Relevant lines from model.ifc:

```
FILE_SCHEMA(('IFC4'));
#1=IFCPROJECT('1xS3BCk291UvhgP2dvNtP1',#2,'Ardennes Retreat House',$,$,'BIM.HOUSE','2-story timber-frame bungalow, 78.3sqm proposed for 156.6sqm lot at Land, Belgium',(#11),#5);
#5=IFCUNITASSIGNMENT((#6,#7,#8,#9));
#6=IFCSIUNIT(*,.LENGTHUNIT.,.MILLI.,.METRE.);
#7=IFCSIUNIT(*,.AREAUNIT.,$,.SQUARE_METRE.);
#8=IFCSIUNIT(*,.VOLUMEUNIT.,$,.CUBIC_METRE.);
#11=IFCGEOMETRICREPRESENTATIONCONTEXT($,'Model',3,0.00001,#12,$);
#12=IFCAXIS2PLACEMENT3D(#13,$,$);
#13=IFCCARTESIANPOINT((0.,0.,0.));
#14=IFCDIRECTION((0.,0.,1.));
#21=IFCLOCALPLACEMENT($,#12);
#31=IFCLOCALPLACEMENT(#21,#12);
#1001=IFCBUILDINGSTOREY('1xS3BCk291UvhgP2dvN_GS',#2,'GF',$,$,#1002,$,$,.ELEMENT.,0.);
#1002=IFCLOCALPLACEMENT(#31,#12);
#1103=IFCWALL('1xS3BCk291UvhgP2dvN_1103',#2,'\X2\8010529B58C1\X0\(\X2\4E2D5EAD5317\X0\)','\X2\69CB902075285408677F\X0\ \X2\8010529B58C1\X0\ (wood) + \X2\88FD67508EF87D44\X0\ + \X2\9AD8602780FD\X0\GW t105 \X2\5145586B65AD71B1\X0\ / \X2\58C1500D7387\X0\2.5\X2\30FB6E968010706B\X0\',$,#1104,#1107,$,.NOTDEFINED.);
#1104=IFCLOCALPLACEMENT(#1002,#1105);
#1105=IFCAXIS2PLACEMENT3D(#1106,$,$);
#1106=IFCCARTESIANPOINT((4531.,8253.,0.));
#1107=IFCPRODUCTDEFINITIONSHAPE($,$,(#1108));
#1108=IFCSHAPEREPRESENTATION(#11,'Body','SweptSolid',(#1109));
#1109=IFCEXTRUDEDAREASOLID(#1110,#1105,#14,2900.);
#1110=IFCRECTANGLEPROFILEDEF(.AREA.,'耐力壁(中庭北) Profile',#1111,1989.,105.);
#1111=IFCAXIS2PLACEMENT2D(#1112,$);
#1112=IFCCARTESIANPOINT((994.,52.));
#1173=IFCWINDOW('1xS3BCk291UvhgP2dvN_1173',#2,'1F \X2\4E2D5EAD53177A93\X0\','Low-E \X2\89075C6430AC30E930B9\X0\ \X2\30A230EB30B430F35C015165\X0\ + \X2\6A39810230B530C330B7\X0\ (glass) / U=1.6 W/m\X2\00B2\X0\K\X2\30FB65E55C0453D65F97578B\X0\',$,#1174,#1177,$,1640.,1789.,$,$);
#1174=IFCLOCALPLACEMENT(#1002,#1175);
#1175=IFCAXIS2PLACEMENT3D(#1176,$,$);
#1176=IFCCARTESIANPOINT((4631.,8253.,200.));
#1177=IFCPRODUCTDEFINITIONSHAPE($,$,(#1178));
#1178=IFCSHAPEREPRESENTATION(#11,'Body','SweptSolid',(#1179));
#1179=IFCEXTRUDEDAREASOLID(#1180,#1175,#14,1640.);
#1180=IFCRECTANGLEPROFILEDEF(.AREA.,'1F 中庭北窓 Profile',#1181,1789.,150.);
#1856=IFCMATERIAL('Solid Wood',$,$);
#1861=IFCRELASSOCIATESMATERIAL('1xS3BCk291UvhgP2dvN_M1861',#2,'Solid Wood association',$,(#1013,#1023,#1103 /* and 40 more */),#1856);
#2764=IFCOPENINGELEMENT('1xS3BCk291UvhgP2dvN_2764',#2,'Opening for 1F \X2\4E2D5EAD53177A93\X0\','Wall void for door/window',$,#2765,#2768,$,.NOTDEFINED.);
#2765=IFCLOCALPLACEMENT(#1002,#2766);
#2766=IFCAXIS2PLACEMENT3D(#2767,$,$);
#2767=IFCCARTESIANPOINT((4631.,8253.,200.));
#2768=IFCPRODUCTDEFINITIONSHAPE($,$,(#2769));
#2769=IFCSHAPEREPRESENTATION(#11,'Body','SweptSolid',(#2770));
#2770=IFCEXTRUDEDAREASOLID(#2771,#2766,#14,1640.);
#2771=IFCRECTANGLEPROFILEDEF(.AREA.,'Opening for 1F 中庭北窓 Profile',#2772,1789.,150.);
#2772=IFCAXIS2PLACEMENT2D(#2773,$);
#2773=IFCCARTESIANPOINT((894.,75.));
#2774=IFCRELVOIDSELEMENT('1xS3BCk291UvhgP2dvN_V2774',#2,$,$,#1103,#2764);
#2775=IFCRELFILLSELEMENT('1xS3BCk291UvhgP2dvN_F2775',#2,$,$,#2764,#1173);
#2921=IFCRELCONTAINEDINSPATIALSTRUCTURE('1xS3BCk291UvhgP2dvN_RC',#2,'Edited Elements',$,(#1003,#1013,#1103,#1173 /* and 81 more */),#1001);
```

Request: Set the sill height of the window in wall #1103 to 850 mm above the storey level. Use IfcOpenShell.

```python
import numpy as np
import ifcopenshell
import ifcopenshell.api.geometry
import ifcopenshell.geom
import ifcopenshell.util.element
import ifcopenshell.util.placement
import ifcopenshell.util.shape
import ifcopenshell.util.unit

model = ifcopenshell.open("model.ifc")
unit_scale = ifcopenshell.util.unit.calculate_unit_scale(model)

window = model.by_guid("1xS3BCk291UvhgP2dvN_1173")
opening = window.FillsVoids[0].RelatingOpeningElement
storey = ifcopenshell.util.element.get_container(window, ifc_class="IfcBuildingStorey")
level = ifcopenshell.util.placement.get_local_placement(storey.ObjectPlacement)[2, 3]

# The opening's origin need not be at the sill, so measure its lowest point.
shape = ifcopenshell.geom.create_shape(ifcopenshell.geom.settings(), opening)
bottom = ifcopenshell.util.shape.get_shape_bottom_elevation(shape, shape.geometry) / unit_scale
dz = level + 0.85 / unit_scale - bottom

shift = np.array([0.0, 0.0, dz])
# The window is not placed relative to its opening, so move both.
for product in (opening, window):
    matrix = ifcopenshell.util.placement.get_local_placement(product.ObjectPlacement)
    matrix[:3, 3] += shift
    ifcopenshell.api.geometry.edit_object_placement(model, product=product, matrix=matrix, is_si=False)

print(f"moved by {dz * unit_scale:+.3f} m")

model.write("model-out.ifc")
```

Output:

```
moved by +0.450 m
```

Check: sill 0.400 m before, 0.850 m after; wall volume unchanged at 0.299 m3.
